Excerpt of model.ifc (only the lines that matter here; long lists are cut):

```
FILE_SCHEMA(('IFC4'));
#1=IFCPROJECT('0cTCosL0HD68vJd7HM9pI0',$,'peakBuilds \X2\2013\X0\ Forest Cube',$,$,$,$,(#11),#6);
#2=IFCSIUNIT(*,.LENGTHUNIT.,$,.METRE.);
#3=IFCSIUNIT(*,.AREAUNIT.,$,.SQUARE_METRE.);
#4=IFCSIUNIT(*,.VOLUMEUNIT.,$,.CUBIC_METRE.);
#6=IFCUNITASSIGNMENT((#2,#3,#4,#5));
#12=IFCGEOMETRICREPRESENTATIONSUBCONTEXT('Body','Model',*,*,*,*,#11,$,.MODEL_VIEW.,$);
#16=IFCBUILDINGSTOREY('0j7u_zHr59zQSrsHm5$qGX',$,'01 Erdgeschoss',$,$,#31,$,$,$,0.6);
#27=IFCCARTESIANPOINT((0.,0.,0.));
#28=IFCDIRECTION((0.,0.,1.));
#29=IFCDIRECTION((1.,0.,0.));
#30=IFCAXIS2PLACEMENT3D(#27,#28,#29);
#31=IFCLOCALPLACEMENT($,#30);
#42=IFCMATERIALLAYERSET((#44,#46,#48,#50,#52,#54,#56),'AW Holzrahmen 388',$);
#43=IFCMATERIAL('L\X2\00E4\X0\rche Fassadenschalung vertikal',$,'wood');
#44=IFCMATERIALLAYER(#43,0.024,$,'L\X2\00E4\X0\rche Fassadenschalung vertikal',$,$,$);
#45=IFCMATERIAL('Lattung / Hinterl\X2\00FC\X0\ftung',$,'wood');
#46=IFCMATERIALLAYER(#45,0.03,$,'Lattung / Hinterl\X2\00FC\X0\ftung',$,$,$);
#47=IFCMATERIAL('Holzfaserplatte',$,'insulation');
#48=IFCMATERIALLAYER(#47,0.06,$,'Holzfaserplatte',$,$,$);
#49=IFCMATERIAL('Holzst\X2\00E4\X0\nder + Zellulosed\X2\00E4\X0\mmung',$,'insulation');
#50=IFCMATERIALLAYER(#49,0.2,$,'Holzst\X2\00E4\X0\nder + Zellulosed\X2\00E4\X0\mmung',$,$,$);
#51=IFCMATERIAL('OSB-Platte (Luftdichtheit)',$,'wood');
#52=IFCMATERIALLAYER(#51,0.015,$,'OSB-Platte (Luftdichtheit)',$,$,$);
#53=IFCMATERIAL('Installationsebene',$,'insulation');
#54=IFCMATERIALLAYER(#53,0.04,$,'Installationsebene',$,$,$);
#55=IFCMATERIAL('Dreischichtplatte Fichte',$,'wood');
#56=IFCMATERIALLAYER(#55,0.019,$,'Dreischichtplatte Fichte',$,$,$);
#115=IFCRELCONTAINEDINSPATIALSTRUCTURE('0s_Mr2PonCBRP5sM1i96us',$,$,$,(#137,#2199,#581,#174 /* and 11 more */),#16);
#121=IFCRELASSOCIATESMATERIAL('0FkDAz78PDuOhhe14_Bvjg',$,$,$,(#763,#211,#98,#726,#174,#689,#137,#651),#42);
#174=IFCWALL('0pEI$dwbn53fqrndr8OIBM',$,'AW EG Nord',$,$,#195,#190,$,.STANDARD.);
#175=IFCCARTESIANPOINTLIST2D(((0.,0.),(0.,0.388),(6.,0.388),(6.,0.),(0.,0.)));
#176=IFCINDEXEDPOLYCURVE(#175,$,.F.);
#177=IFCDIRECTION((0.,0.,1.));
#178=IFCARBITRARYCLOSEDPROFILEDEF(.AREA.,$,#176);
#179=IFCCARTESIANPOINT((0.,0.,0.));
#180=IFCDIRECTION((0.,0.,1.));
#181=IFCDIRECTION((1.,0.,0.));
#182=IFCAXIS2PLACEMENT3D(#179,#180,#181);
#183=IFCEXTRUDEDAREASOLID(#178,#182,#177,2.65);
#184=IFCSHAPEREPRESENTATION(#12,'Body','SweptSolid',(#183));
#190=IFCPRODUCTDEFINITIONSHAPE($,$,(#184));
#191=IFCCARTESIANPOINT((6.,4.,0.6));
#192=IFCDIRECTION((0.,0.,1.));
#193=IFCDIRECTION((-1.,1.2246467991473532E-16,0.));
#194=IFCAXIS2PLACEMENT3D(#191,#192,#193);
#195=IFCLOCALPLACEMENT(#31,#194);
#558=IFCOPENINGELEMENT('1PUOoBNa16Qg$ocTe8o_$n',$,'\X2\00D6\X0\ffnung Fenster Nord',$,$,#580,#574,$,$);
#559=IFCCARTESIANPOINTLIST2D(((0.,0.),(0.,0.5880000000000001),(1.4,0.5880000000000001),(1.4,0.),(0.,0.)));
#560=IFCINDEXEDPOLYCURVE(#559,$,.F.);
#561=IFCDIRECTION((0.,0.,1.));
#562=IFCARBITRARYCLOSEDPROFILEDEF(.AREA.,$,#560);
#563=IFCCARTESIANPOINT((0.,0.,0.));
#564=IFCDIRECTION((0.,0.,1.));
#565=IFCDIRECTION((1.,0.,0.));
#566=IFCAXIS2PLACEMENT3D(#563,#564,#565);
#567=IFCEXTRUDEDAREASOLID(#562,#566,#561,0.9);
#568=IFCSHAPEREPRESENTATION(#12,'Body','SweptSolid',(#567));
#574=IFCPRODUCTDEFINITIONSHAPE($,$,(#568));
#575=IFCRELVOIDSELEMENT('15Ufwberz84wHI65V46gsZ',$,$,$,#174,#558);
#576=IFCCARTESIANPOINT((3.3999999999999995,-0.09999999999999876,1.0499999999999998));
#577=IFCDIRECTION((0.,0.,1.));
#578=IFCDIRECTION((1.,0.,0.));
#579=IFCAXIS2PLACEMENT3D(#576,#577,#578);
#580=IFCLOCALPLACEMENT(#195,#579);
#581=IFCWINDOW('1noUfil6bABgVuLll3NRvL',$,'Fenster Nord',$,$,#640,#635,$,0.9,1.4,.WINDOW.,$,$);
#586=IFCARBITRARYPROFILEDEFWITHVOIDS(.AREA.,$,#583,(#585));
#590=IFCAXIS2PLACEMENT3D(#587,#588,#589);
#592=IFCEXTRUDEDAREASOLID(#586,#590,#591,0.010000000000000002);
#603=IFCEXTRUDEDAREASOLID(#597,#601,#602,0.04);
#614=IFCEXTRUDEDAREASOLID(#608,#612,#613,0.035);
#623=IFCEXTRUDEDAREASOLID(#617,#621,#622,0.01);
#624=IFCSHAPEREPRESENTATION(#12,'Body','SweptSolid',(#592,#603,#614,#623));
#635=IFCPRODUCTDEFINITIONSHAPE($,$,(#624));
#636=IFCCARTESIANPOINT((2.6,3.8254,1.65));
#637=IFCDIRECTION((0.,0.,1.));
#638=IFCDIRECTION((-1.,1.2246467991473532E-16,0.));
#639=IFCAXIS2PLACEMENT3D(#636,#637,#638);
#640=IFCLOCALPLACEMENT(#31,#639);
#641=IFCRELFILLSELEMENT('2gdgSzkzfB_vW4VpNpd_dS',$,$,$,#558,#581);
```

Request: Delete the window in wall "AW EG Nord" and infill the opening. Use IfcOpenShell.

```python
import ifcopenshell
import ifcopenshell.api.feature
import ifcopenshell.api.root
import ifcopenshell.geom
import ifcopenshell.util.shape

model = ifcopenshell.open("model.ifc")
settings = ifcopenshell.geom.settings()


def volume(element):
    """Net volume in cubic metres, openings subtracted."""
    shape = ifcopenshell.geom.create_shape(settings, element)
    return ifcopenshell.util.shape.get_volume(shape.geometry)


window = model.by_guid("1noUfil6bABgVuLll3NRvL")
opening = window.FillsVoids[0].RelatingOpeningElement
wall = opening.VoidsElements[0].RelatingBuildingElement
before = volume(wall)

ifcopenshell.api.root.remove_product(model, product=window)
ifcopenshell.api.feature.remove_feature(model, feature=opening)

after = volume(wall)

print(f"wall volume {before:.3f} -> {after:.3f} m3")

model.write("model_updated.ifc")
```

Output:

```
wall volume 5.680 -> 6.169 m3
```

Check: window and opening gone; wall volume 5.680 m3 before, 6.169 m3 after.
